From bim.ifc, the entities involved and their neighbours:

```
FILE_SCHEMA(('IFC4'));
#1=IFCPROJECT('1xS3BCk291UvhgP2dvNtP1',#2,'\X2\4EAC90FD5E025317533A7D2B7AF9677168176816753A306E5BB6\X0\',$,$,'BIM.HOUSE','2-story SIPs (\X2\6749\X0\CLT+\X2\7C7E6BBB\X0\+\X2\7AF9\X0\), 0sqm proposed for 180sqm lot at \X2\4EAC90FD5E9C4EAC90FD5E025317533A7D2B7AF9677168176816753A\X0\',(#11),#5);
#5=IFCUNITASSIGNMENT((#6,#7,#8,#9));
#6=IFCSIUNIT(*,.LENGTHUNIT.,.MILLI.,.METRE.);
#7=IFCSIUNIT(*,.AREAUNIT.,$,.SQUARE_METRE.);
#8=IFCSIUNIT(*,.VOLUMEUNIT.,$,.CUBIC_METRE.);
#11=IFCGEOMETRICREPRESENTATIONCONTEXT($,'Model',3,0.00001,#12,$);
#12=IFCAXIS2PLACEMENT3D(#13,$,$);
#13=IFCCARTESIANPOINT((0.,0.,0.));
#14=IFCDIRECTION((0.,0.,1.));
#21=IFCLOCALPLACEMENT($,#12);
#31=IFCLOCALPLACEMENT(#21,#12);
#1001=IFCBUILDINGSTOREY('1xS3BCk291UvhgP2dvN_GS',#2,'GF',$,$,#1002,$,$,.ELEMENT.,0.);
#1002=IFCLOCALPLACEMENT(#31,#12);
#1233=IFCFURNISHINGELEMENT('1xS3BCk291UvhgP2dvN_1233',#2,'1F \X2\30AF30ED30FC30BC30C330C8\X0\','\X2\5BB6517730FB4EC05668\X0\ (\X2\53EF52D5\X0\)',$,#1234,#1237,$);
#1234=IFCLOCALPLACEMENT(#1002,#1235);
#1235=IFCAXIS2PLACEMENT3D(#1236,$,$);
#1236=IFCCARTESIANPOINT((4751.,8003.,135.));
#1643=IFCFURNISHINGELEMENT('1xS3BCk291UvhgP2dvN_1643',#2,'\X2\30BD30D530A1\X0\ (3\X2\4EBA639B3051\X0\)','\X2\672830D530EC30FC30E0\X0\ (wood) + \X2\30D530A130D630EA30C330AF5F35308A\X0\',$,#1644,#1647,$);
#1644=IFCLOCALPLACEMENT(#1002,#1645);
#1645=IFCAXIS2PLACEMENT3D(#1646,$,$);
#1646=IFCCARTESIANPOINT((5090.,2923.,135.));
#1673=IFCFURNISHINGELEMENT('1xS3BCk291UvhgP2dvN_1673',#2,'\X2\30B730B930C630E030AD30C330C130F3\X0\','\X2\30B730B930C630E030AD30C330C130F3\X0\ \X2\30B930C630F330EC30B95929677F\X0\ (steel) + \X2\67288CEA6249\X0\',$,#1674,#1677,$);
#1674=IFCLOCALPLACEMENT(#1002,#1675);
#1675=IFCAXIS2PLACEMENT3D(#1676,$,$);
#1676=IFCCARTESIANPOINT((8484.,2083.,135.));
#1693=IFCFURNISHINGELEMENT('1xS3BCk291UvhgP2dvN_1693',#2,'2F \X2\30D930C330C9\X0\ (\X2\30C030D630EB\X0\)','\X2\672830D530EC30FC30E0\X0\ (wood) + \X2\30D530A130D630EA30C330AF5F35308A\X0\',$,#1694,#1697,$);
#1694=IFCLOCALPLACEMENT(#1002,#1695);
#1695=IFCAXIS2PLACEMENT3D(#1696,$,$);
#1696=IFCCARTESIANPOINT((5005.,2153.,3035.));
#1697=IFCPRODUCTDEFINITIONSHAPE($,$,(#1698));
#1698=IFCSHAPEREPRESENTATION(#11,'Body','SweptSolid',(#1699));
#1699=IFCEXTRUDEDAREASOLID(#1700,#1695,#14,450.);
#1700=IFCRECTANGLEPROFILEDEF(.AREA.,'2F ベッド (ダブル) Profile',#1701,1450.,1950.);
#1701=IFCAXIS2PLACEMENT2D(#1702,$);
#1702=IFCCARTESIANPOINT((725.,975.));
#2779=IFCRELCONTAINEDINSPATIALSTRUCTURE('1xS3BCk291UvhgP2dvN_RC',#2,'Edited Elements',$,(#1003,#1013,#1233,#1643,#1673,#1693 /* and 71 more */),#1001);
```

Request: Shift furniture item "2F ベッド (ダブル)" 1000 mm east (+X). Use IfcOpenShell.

```python
import ifcopenshell
import ifcopenshell.api.geometry
import ifcopenshell.util.placement

model = ifcopenshell.open("bim.ifc")

item = model.by_guid("1xS3BCk291UvhgP2dvN_1693")
matrix = ifcopenshell.util.placement.get_local_placement(item.ObjectPlacement)
matrix[0, 3] += 1000.0
ifcopenshell.api.geometry.edit_object_placement(model, product=item, matrix=matrix, is_si=False)

print(ifcopenshell.util.placement.get_local_placement(item.ObjectPlacement).round(3) + 0.0)

model.write("bim-out.ifc")
```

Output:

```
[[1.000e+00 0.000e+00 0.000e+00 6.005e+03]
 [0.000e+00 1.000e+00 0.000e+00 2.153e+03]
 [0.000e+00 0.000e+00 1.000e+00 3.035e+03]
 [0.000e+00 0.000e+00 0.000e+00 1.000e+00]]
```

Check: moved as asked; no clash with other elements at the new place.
